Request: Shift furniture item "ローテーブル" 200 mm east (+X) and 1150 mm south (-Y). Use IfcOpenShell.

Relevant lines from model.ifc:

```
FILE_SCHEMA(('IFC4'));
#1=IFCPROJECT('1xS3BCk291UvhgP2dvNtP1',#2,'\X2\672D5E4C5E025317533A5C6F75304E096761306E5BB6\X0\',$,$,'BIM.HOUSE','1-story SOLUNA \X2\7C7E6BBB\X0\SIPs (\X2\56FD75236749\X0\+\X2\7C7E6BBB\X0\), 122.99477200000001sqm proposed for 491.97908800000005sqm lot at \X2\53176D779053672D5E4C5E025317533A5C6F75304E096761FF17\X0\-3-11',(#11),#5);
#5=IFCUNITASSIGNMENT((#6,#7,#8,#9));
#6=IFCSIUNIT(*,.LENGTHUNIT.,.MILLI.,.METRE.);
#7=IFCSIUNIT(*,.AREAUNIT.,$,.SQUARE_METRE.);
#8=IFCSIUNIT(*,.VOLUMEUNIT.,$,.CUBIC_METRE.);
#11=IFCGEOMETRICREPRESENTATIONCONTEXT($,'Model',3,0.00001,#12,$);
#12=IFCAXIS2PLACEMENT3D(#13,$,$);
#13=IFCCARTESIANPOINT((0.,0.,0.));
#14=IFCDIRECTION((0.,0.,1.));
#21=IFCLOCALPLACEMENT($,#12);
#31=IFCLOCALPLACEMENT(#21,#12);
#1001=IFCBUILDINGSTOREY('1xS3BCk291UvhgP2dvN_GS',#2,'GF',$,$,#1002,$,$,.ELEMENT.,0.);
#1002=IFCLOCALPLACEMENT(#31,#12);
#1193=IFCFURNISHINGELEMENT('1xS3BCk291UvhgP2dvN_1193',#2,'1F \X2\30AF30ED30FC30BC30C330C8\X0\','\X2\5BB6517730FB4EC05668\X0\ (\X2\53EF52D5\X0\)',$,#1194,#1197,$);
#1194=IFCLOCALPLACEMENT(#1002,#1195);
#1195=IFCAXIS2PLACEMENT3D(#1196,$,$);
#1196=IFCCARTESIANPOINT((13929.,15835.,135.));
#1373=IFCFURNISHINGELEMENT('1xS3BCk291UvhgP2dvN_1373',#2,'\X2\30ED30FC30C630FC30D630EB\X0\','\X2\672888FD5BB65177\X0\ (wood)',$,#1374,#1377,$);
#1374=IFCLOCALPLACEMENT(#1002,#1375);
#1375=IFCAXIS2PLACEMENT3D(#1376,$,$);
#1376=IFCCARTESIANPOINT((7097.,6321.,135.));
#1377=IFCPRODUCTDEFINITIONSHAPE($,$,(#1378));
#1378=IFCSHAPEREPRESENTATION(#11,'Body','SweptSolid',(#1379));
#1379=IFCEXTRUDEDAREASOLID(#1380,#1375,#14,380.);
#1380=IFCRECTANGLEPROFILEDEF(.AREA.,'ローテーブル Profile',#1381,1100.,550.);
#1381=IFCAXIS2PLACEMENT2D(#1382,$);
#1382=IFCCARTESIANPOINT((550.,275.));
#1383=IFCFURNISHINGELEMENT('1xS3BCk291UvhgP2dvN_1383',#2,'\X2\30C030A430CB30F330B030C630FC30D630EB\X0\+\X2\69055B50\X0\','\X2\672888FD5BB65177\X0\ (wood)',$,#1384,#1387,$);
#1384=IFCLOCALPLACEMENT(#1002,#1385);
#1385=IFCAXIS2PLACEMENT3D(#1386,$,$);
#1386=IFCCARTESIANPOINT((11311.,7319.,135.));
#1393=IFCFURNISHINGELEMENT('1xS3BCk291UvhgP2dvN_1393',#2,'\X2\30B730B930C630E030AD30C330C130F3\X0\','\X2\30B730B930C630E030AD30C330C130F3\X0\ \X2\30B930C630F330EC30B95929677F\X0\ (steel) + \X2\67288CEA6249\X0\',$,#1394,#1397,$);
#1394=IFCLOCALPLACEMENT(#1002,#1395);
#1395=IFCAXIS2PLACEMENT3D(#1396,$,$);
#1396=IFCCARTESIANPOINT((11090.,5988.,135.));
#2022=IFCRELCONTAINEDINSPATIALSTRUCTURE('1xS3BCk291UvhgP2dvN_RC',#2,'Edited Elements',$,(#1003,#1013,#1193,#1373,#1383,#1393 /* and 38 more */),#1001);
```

```python
import ifcopenshell
import ifcopenshell.api.geometry
import ifcopenshell.util.placement

model = ifcopenshell.open("model.ifc")

item = model.by_guid("1xS3BCk291UvhgP2dvN_1373")
matrix = ifcopenshell.util.placement.get_local_placement(item.ObjectPlacement)
matrix[0, 3] += 200.0
matrix[1, 3] -= 1150.0
ifcopenshell.api.geometry.edit_object_placement(model, product=item, matrix=matrix, is_si=False)

print(ifcopenshell.util.placement.get_local_placement(item.ObjectPlacement).round(3) + 0.0)

model.write("model_edited.ifc")
```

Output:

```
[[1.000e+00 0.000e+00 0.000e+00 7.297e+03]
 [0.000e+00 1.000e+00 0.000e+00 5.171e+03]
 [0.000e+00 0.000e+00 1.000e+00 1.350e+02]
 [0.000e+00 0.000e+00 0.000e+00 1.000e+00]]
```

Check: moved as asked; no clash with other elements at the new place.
